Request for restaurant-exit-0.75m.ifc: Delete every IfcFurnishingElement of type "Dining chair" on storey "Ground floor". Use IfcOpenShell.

First a look at what the model holds.

```python
import ifcopenshell
import ifcopenshell.util.element

model = ifcopenshell.open("restaurant-exit-0.75m.ifc")
print(model.schema)
storey = next(s for s in model.by_type("IfcBuildingStorey") if s.Name == "Ground floor")
furniture = [e for e in ifcopenshell.util.element.get_decomposition(storey) if e.is_a("IfcFurnishingElement")]
seen = {}
for e in furniture:
    element_type = ifcopenshell.util.element.get_type(e)
    name = element_type.Name if element_type not in (None, e) else None
    seen[name] = seen.get(name, 0) + 1
for name, count in sorted(seen.items(), key=str):
    print(count, "x", name)
```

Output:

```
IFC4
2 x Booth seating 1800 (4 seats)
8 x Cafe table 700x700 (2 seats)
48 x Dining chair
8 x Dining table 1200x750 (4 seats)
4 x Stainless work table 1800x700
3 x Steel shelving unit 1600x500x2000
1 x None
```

```python
import ifcopenshell
import ifcopenshell.api.root
import ifcopenshell.util.element

model = ifcopenshell.open("restaurant-exit-0.75m.ifc")

storey = next(s for s in model.by_type("IfcBuildingStorey") if s.Name == "Ground floor")
furniture = [e for e in ifcopenshell.util.element.get_decomposition(storey) if e.is_a("IfcFurnishingElement")]
targets = [e for e in furniture if (t := ifcopenshell.util.element.get_type(e)) not in (None, e) and t.Name == "Dining chair"]

for e in targets:
    ifcopenshell.api.root.remove_product(model, product=e)
print(len(targets), "removed")

model.write("restaurant-exit-0.75m_edited.ifc")
```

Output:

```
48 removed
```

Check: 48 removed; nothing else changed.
